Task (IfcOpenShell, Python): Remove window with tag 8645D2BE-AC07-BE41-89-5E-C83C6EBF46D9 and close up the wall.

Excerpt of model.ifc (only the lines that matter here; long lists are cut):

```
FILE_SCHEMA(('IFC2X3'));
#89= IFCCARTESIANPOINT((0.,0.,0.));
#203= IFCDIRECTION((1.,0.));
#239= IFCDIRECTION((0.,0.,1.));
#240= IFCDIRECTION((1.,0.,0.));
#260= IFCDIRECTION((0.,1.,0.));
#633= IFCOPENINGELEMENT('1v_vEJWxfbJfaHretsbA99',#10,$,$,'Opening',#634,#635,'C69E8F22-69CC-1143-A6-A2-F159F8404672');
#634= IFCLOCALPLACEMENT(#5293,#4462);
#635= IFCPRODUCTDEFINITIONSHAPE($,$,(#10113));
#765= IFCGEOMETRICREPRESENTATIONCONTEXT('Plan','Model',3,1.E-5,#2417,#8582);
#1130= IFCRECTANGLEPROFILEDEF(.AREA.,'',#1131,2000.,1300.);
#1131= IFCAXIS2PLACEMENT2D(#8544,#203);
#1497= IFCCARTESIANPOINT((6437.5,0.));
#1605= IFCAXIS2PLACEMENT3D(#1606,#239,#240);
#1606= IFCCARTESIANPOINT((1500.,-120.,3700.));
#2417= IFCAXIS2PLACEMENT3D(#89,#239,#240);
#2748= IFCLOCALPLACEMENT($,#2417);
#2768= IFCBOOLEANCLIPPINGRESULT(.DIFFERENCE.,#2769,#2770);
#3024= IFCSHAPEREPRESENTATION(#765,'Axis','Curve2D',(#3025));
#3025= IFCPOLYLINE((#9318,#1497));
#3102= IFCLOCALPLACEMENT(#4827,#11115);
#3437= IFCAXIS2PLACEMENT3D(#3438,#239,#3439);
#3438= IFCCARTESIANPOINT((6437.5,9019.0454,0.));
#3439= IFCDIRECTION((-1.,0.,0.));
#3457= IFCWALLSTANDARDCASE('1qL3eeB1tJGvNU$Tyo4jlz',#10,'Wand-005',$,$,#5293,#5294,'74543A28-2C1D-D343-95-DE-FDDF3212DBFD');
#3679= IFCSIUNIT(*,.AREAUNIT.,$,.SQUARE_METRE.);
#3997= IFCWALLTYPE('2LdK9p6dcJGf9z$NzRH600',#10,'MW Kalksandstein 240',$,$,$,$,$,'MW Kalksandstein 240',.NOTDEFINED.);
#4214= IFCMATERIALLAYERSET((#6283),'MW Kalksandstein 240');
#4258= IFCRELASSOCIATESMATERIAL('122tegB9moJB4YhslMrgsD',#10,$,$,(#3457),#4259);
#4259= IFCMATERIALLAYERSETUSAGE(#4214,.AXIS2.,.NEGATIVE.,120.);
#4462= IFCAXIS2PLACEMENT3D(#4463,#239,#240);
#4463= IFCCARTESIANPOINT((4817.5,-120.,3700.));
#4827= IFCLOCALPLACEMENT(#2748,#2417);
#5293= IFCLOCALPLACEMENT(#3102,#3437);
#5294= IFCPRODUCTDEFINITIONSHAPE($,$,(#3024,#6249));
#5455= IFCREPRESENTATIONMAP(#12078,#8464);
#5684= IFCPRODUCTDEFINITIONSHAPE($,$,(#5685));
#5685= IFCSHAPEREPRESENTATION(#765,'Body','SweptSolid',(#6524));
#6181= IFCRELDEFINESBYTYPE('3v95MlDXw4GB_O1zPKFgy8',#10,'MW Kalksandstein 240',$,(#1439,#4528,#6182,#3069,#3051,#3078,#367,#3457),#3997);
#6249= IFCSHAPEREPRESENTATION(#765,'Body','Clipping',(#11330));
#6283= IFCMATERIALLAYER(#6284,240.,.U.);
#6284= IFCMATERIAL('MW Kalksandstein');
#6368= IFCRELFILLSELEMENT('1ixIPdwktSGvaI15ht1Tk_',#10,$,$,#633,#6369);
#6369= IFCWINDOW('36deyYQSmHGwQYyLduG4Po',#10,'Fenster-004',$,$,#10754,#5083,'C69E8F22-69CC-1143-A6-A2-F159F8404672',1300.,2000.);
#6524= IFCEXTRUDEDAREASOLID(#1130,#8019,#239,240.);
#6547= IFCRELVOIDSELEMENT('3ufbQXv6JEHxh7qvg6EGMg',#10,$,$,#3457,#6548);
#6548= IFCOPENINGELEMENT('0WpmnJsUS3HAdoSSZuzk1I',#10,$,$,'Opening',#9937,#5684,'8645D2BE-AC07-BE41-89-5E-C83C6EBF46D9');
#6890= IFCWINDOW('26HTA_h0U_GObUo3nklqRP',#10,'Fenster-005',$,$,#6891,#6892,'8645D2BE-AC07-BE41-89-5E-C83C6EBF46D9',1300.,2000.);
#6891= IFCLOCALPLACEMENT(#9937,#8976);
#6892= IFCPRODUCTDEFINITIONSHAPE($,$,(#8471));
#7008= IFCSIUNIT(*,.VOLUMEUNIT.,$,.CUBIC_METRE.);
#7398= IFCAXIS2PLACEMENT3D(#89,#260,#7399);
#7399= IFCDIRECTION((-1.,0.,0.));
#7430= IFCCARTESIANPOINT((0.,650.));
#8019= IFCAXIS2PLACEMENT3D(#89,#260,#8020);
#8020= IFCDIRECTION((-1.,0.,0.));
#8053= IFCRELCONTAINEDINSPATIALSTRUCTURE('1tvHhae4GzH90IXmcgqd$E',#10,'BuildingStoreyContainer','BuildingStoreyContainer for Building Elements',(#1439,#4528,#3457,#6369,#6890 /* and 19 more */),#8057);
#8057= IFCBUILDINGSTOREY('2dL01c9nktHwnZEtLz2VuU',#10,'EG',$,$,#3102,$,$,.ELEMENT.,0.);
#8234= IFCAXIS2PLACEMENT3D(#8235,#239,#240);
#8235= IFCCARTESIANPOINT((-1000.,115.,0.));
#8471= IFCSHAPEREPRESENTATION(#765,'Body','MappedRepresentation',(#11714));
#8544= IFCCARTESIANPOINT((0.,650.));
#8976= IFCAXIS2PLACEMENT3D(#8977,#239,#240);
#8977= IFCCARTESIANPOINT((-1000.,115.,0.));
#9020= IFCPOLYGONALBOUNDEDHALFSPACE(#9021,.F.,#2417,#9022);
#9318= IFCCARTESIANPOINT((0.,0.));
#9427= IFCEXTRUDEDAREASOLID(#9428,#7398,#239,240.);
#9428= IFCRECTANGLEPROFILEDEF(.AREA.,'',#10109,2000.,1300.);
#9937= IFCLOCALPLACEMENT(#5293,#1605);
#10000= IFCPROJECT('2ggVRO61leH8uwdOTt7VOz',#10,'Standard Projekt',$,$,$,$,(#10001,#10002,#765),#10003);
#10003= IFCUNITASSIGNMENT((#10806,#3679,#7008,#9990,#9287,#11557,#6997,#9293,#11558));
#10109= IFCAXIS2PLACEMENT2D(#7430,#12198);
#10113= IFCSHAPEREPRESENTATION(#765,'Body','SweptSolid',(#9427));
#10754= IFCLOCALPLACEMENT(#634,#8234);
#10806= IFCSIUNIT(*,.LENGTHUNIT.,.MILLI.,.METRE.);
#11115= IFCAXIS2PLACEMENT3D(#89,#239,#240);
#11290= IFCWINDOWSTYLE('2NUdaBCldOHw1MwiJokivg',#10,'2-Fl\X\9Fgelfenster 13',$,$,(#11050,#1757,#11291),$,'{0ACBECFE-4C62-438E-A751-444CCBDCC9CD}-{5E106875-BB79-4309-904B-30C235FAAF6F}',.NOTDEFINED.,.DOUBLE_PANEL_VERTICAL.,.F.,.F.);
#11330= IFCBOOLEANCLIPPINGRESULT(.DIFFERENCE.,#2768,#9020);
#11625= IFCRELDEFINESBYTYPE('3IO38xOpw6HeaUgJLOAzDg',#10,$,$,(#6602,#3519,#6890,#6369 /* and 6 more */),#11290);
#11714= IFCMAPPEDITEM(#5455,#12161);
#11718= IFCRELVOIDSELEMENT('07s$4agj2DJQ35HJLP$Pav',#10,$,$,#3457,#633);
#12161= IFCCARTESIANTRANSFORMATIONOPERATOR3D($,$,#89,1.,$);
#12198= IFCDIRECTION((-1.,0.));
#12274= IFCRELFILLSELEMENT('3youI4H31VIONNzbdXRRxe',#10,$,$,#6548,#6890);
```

```python
import ifcopenshell
import ifcopenshell.api.feature
import ifcopenshell.api.root
import ifcopenshell.geom
import ifcopenshell.util.shape

model = ifcopenshell.open("model.ifc")
settings = ifcopenshell.geom.settings()


def volume(element):
    """Net volume in cubic metres, openings subtracted."""
    shape = ifcopenshell.geom.create_shape(settings, element)
    return ifcopenshell.util.shape.get_volume(shape.geometry)


window = model.by_id(6890)
opening = window.FillsVoids[0].RelatingOpeningElement
wall = opening.VoidsElements[0].RelatingBuildingElement
before = volume(wall)

ifcopenshell.api.root.remove_product(model, product=window)
ifcopenshell.api.feature.remove_feature(model, feature=opening)

after = volume(wall)

print(f"wall volume {before:.3f} -> {after:.3f} m3")

model.write("model_v2.ifc")
```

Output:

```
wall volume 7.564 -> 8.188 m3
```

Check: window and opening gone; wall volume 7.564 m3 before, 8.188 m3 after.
